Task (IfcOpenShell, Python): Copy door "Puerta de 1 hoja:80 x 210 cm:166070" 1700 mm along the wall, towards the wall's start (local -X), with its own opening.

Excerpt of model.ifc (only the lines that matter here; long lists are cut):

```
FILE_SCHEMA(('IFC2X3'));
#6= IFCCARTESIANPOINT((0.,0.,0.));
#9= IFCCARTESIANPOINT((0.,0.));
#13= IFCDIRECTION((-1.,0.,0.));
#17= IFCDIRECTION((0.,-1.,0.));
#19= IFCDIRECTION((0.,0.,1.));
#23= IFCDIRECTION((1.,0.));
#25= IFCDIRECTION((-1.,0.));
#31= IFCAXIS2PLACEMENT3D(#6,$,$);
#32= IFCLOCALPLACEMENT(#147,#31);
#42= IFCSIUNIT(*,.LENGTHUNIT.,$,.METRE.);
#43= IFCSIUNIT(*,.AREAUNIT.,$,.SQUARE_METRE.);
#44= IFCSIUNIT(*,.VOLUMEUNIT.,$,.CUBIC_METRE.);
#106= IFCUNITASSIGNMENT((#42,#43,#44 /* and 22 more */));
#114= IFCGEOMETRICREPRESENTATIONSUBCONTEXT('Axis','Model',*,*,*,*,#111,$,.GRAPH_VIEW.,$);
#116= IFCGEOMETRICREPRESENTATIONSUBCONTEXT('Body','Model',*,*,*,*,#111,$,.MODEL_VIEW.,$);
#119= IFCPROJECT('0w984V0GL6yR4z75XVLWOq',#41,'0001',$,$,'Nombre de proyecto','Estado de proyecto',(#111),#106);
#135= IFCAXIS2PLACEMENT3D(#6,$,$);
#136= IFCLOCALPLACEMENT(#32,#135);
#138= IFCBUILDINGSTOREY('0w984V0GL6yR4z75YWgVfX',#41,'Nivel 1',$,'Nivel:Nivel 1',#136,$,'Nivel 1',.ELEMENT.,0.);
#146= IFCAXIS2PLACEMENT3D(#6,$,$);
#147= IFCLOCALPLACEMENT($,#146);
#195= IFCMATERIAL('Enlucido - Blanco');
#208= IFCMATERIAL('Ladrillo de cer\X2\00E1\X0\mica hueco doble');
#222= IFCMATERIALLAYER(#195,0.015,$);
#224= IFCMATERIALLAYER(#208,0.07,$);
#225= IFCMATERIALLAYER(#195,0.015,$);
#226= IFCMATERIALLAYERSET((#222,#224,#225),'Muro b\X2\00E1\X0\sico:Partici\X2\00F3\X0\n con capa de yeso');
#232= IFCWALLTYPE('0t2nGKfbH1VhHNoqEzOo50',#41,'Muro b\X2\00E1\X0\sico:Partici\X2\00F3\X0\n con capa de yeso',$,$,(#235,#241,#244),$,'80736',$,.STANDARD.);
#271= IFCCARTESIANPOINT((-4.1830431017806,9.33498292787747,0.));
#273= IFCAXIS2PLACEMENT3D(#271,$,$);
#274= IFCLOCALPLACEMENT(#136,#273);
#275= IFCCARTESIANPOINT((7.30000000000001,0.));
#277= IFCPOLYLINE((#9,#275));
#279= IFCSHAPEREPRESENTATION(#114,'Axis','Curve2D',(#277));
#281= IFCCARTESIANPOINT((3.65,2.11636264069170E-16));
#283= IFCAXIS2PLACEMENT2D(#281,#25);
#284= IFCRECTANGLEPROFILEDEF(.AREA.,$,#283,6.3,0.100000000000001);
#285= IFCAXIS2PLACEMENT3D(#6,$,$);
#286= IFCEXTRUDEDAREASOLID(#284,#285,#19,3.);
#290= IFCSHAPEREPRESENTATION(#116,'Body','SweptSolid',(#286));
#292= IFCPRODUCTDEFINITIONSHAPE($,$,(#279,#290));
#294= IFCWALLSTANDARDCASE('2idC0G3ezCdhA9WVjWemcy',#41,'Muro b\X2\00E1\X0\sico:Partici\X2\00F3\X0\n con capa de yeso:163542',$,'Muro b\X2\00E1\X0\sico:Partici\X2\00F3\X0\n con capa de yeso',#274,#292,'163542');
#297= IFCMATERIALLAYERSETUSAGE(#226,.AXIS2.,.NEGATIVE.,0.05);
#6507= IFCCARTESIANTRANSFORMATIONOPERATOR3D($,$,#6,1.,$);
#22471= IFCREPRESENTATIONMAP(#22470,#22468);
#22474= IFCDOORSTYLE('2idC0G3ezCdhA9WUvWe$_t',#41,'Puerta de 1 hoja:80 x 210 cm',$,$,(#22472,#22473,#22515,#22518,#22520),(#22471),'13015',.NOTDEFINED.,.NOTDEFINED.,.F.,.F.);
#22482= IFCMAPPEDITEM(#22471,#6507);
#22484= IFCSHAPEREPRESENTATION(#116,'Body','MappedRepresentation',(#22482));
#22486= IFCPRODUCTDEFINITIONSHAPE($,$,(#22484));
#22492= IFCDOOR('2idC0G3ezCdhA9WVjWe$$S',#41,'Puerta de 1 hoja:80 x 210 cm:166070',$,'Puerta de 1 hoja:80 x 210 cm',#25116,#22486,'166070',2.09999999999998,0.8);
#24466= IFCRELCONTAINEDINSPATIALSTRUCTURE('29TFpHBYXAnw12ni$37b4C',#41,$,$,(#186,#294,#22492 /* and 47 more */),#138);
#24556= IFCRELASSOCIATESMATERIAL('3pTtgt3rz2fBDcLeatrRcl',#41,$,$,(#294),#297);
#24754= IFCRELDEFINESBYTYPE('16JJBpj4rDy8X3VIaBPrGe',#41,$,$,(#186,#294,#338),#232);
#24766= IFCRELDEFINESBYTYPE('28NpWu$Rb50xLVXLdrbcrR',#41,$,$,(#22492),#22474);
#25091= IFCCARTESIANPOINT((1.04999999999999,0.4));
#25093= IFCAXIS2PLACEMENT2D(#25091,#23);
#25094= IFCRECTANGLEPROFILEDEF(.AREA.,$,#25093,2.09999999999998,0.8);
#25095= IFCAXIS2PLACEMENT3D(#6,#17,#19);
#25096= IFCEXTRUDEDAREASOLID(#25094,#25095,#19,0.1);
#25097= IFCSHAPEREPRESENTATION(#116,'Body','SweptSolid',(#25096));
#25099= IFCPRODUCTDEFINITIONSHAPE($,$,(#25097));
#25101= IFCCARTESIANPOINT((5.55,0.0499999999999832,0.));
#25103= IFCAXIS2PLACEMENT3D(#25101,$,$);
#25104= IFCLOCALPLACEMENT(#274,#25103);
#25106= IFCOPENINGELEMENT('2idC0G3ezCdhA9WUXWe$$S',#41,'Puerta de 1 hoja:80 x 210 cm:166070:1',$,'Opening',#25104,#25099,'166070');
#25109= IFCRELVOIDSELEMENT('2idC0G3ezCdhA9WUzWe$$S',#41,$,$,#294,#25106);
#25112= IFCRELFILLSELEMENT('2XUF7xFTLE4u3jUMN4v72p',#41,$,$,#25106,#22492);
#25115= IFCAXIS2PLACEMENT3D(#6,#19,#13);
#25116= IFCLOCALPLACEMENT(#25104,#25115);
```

```python
import ifcopenshell
import ifcopenshell.api.feature
import ifcopenshell.api.geometry
import ifcopenshell.api.root
import ifcopenshell.geom
import ifcopenshell.util.element
import ifcopenshell.util.placement
import ifcopenshell.util.shape

model = ifcopenshell.open("model.ifc")
settings = ifcopenshell.geom.settings()


def volume(element):
    """Net volume in cubic metres, openings subtracted."""
    shape = ifcopenshell.geom.create_shape(settings, element)
    return ifcopenshell.util.shape.get_volume(shape.geometry)


def reuse_history(source, copy):
    """copy_class also copies each property set's owner history, people and application; keep the originals."""
    for rel in copy.IsDefinedBy:
        if rel.is_a("IfcRelDefinesByProperties") and (history := rel.RelatingPropertyDefinition.OwnerHistory):
            rel.RelatingPropertyDefinition.OwnerHistory = source.OwnerHistory
            ifcopenshell.util.element.remove_deep2(model, history)


door = model.by_id(22492)
opening = door.FillsVoids[0].RelatingOpeningElement
wall = opening.VoidsElements[0].RelatingBuildingElement
before = volume(wall)
shift = ifcopenshell.util.placement.get_local_placement(wall.ObjectPlacement)[:3, 0] * -1.7

# copy_class copies the void relationship, type, container and properties, but no geometry.
new_opening = ifcopenshell.api.root.copy_class(model, product=opening)
new_opening.Representation = ifcopenshell.util.element.copy_deep(
    model, opening.Representation, exclude=["IfcGeometricRepresentationContext", "IfcRepresentationMap"]
)
new_opening.Name = "Puerta de 1 hoja:80 x 210 cm"
new_opening.Tag = None
new_door = ifcopenshell.api.root.copy_class(model, product=door)
new_door.Representation = ifcopenshell.util.element.copy_deep(
    model, door.Representation, exclude=["IfcGeometricRepresentationContext", "IfcRepresentationMap"]
)
new_door.Name = "Puerta de 1 hoja:80 x 210 cm"
new_door.Tag = None
reuse_history(door, new_door)
fills = ifcopenshell.api.feature.add_filling(model, opening=new_opening, element=new_door)
fills.OwnerHistory = new_door.OwnerHistory  # required in IFC2X3

for old, new in ((opening, new_opening), (door, new_door)):
    matrix = ifcopenshell.util.placement.get_local_placement(old.ObjectPlacement)
    matrix[:3, 3] += shift
    ifcopenshell.api.geometry.edit_object_placement(model, product=new, matrix=matrix, is_si=False)

after = volume(wall)

print(f"wall volume {before:.3f} -> {after:.3f} m3")

model.write("model_rev.ifc")
```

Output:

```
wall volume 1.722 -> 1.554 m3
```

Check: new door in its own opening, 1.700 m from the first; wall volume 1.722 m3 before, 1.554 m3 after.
